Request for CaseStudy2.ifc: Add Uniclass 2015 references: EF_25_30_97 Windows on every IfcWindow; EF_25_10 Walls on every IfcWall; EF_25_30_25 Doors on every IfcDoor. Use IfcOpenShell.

First a look at what the model holds.

```python
import ifcopenshell

model = ifcopenshell.open("CaseStudy2.ifc")
print(model.schema)
print("classifications:", [c.Name for c in model.by_type("IfcClassification")])
for ifc_class in ("IfcDoor", "IfcRoof", "IfcStair", "IfcWall", "IfcWindow"):
    print(ifc_class, len(model.by_type(ifc_class)))
```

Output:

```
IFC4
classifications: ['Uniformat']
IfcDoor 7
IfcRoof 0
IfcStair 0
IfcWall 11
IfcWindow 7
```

```python
import ifcopenshell
import ifcopenshell.api.classification

model = ifcopenshell.open("CaseStudy2.ifc")

system = ifcopenshell.api.classification.add_classification(model, classification="Uniclass 2015")

codes = {
    "IfcWindow": ("EF_25_30_97", "Windows"),
    "IfcWall": ("EF_25_10", "Walls"),
    "IfcDoor": ("EF_25_30_25", "Doors"),
}
for ifc_class, (code, name) in codes.items():
    products = model.by_type(ifc_class)
    ifcopenshell.api.classification.add_reference(
        model, products=products, classification=system, identification=code, name=name
    )
    print(code, len(products))

model.write("CaseStudy2_edited.ifc")
```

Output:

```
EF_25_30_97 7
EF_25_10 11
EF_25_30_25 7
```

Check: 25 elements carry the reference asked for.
